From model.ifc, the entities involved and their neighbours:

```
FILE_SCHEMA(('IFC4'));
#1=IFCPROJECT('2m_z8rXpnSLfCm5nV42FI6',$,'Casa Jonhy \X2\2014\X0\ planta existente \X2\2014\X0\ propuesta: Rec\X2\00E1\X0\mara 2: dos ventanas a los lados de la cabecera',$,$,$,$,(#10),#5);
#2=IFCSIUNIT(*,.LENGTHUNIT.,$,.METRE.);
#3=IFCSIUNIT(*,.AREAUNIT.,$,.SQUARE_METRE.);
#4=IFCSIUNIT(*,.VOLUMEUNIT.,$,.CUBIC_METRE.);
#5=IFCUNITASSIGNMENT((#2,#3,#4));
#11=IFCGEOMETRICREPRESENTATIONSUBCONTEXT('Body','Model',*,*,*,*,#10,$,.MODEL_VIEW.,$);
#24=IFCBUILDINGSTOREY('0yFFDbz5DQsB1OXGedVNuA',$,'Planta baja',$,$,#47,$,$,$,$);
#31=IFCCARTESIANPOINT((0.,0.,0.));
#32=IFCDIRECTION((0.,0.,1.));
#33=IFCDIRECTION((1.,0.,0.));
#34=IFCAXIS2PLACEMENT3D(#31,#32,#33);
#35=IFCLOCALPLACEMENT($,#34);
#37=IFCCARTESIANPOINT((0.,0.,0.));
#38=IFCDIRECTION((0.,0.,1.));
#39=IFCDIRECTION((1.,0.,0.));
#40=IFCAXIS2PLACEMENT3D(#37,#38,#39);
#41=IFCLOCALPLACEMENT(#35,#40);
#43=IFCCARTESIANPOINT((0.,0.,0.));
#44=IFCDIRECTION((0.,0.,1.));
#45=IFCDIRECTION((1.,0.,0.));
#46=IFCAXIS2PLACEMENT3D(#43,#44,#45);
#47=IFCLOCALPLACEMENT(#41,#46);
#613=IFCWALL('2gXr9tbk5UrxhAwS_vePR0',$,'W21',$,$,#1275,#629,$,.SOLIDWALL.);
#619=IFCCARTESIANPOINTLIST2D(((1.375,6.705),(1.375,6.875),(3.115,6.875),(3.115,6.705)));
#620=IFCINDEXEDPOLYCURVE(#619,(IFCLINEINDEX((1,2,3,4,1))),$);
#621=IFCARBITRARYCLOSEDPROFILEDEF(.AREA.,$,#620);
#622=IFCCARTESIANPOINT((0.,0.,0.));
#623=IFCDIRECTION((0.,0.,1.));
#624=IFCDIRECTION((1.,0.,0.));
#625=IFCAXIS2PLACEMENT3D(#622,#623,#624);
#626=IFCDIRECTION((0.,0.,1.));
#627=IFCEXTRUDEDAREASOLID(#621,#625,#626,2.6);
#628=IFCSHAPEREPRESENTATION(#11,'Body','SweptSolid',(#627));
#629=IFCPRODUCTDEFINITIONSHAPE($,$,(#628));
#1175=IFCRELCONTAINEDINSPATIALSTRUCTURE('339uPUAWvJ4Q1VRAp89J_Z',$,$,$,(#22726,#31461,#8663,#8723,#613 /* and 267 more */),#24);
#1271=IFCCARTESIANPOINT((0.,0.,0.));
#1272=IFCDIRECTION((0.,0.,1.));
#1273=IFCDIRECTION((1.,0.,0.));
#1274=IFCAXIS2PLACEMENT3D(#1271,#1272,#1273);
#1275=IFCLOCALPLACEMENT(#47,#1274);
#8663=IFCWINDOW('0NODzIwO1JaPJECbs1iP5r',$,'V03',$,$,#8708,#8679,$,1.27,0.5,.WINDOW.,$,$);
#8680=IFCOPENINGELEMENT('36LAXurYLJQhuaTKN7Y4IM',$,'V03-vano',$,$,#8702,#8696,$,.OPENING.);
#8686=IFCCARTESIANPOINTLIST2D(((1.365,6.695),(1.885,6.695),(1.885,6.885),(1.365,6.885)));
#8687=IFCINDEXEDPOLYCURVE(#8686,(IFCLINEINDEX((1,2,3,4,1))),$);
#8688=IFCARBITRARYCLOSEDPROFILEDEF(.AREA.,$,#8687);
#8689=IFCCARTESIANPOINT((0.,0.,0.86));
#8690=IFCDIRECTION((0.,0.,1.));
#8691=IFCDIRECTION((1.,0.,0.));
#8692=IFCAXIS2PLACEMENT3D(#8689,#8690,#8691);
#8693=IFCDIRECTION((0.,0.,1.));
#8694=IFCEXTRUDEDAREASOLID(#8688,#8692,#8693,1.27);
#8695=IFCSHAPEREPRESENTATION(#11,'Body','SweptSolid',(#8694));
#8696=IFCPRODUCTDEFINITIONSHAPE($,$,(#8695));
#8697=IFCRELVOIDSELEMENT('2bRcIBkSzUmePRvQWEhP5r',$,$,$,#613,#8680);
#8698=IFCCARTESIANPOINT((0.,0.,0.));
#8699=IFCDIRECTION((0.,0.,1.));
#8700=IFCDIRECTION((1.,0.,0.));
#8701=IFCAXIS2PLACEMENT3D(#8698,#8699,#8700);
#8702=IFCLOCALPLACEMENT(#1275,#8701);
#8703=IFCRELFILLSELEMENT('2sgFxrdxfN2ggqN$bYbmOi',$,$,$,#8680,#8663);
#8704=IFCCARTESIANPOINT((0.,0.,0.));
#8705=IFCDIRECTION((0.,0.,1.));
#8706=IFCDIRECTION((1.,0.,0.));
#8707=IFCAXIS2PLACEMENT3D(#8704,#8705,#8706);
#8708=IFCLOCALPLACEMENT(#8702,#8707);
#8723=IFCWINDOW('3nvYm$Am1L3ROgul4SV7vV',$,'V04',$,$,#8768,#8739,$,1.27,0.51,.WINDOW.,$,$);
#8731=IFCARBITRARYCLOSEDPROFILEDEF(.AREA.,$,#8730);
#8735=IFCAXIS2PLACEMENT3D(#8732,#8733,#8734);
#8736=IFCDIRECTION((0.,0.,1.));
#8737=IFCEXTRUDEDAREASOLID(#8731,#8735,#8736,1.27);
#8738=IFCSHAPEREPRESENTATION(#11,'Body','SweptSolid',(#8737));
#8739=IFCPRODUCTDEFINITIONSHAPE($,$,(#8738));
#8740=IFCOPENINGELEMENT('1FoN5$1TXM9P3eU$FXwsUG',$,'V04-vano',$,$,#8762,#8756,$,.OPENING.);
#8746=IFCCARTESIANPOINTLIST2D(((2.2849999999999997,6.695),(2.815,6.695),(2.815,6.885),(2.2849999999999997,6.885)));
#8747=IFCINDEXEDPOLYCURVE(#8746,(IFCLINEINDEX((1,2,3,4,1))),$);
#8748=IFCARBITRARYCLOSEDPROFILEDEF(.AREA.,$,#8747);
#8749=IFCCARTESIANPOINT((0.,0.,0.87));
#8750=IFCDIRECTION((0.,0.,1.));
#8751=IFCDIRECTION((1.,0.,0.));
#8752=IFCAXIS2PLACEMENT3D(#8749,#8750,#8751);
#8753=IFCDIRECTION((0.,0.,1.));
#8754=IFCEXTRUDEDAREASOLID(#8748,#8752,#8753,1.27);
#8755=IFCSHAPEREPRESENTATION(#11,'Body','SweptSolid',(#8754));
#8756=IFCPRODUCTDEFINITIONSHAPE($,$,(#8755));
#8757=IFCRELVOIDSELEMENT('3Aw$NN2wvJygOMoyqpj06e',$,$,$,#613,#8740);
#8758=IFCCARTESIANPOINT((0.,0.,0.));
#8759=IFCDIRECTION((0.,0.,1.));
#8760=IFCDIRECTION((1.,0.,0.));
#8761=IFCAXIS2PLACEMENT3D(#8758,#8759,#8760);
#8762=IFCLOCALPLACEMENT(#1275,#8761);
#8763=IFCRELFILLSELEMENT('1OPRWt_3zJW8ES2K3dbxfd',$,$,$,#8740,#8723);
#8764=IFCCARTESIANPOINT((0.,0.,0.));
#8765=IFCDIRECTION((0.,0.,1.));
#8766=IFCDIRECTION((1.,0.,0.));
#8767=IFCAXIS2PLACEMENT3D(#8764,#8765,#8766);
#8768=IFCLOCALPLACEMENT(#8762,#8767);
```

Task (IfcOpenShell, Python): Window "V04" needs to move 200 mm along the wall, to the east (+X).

```python
import ifcopenshell
import ifcopenshell.api.geometry
import ifcopenshell.util.placement

model = ifcopenshell.open("model.ifc")

window = model.by_guid("3nvYm$Am1L3ROgul4SV7vV")
opening = window.FillsVoids[0].RelatingOpeningElement
wall = opening.VoidsElements[0].RelatingBuildingElement

wall_matrix = ifcopenshell.util.placement.get_local_placement(wall.ObjectPlacement)
shift = wall_matrix[:3, 0] * 0.2
before = ifcopenshell.util.placement.get_local_placement(window.ObjectPlacement)[:3, 3].copy()

# The window is placed relative to its opening, so it follows when the opening moves.
matrix = ifcopenshell.util.placement.get_local_placement(opening.ObjectPlacement)
matrix[:3, 3] += shift
ifcopenshell.api.geometry.edit_object_placement(
    model, product=opening, matrix=matrix, is_si=False, should_transform_children=True
)

after = ifcopenshell.util.placement.get_local_placement(window.ObjectPlacement)[:3, 3]
print("window moved by", (after - before).round(3) + 0.0)

model.write("model_rev.ifc")
```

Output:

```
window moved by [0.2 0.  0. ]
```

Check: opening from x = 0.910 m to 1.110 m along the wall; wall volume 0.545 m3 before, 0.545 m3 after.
